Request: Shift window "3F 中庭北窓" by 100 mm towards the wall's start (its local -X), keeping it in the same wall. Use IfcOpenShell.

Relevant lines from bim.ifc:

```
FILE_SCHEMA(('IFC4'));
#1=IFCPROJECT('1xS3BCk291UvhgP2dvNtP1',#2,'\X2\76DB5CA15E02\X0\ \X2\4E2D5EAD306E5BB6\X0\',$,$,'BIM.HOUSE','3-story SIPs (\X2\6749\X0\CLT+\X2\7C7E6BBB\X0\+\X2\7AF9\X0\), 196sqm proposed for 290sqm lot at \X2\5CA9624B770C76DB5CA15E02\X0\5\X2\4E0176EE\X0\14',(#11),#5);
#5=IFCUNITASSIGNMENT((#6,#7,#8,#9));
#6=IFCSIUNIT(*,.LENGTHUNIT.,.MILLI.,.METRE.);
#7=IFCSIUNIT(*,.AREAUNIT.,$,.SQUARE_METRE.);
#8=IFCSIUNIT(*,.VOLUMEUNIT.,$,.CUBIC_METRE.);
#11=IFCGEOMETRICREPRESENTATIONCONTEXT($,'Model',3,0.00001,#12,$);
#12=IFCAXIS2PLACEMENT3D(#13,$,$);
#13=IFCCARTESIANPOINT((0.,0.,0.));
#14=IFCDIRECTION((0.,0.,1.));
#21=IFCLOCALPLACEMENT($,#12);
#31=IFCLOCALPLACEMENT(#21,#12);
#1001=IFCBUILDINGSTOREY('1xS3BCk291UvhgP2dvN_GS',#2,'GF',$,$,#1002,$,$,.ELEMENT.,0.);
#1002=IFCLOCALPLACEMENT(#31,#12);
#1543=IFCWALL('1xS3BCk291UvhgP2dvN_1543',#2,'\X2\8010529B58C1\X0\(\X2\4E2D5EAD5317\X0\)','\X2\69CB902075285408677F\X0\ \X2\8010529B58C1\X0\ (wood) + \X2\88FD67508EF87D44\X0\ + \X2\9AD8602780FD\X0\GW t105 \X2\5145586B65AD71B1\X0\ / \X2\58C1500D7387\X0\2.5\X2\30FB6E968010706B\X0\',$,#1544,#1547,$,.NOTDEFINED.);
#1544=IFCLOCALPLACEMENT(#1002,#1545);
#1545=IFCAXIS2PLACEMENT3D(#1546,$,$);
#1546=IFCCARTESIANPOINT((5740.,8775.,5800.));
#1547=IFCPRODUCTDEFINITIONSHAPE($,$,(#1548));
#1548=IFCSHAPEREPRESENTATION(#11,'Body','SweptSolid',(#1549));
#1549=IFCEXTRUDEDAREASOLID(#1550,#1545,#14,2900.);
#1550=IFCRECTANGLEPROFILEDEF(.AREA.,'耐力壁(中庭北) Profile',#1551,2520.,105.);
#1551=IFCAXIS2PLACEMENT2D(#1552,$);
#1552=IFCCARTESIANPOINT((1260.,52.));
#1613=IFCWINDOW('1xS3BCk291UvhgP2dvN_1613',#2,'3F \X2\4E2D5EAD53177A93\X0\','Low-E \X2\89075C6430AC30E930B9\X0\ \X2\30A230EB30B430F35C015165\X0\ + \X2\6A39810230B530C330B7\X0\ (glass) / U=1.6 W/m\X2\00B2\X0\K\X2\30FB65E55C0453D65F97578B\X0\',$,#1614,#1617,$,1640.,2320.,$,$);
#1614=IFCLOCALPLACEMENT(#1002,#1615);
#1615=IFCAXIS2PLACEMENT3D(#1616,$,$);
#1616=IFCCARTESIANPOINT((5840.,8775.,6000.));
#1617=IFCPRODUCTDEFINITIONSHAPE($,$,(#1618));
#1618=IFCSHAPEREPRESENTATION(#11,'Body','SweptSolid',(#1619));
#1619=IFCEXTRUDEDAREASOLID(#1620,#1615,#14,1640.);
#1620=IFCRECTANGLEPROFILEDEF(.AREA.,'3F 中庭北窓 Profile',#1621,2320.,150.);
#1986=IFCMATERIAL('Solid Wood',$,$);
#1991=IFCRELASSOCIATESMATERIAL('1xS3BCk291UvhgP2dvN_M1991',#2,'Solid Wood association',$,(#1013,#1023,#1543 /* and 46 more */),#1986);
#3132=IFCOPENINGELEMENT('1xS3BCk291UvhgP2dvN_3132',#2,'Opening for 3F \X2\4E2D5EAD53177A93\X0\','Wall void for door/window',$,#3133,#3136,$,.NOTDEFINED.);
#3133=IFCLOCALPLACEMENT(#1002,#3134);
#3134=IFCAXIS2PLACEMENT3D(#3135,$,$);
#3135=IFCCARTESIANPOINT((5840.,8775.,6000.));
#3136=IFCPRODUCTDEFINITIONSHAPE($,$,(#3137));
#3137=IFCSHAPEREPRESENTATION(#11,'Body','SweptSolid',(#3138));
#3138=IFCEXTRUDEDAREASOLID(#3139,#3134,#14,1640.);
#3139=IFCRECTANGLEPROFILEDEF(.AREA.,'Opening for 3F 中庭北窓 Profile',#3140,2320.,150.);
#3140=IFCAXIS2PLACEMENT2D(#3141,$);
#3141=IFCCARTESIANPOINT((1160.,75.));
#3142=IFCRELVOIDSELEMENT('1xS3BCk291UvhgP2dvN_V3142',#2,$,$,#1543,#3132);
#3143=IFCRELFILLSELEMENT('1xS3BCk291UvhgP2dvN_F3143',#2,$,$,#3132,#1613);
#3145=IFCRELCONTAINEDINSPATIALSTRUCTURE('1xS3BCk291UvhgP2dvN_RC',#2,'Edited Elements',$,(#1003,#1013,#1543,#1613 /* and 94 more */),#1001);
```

```python
import ifcopenshell
import ifcopenshell.api.geometry
import ifcopenshell.util.placement

model = ifcopenshell.open("bim.ifc")

window = model.by_id(1613)
opening = window.FillsVoids[0].RelatingOpeningElement
wall = opening.VoidsElements[0].RelatingBuildingElement

wall_matrix = ifcopenshell.util.placement.get_local_placement(wall.ObjectPlacement)
shift = wall_matrix[:3, 0] * -100.0
before = ifcopenshell.util.placement.get_local_placement(window.ObjectPlacement)[:3, 3].copy()

# The window is not placed relative to its opening, so move both.
for product in (opening, window):
    matrix = ifcopenshell.util.placement.get_local_placement(product.ObjectPlacement)
    matrix[:3, 3] += shift
    ifcopenshell.api.geometry.edit_object_placement(model, product=product, matrix=matrix, is_si=False)

after = ifcopenshell.util.placement.get_local_placement(window.ObjectPlacement)[:3, 3]
print("window moved by", (after - before).round(3) + 0.0)

model.write("bim_edited.ifc")
```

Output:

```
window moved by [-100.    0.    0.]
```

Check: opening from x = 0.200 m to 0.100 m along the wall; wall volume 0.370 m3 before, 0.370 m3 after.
